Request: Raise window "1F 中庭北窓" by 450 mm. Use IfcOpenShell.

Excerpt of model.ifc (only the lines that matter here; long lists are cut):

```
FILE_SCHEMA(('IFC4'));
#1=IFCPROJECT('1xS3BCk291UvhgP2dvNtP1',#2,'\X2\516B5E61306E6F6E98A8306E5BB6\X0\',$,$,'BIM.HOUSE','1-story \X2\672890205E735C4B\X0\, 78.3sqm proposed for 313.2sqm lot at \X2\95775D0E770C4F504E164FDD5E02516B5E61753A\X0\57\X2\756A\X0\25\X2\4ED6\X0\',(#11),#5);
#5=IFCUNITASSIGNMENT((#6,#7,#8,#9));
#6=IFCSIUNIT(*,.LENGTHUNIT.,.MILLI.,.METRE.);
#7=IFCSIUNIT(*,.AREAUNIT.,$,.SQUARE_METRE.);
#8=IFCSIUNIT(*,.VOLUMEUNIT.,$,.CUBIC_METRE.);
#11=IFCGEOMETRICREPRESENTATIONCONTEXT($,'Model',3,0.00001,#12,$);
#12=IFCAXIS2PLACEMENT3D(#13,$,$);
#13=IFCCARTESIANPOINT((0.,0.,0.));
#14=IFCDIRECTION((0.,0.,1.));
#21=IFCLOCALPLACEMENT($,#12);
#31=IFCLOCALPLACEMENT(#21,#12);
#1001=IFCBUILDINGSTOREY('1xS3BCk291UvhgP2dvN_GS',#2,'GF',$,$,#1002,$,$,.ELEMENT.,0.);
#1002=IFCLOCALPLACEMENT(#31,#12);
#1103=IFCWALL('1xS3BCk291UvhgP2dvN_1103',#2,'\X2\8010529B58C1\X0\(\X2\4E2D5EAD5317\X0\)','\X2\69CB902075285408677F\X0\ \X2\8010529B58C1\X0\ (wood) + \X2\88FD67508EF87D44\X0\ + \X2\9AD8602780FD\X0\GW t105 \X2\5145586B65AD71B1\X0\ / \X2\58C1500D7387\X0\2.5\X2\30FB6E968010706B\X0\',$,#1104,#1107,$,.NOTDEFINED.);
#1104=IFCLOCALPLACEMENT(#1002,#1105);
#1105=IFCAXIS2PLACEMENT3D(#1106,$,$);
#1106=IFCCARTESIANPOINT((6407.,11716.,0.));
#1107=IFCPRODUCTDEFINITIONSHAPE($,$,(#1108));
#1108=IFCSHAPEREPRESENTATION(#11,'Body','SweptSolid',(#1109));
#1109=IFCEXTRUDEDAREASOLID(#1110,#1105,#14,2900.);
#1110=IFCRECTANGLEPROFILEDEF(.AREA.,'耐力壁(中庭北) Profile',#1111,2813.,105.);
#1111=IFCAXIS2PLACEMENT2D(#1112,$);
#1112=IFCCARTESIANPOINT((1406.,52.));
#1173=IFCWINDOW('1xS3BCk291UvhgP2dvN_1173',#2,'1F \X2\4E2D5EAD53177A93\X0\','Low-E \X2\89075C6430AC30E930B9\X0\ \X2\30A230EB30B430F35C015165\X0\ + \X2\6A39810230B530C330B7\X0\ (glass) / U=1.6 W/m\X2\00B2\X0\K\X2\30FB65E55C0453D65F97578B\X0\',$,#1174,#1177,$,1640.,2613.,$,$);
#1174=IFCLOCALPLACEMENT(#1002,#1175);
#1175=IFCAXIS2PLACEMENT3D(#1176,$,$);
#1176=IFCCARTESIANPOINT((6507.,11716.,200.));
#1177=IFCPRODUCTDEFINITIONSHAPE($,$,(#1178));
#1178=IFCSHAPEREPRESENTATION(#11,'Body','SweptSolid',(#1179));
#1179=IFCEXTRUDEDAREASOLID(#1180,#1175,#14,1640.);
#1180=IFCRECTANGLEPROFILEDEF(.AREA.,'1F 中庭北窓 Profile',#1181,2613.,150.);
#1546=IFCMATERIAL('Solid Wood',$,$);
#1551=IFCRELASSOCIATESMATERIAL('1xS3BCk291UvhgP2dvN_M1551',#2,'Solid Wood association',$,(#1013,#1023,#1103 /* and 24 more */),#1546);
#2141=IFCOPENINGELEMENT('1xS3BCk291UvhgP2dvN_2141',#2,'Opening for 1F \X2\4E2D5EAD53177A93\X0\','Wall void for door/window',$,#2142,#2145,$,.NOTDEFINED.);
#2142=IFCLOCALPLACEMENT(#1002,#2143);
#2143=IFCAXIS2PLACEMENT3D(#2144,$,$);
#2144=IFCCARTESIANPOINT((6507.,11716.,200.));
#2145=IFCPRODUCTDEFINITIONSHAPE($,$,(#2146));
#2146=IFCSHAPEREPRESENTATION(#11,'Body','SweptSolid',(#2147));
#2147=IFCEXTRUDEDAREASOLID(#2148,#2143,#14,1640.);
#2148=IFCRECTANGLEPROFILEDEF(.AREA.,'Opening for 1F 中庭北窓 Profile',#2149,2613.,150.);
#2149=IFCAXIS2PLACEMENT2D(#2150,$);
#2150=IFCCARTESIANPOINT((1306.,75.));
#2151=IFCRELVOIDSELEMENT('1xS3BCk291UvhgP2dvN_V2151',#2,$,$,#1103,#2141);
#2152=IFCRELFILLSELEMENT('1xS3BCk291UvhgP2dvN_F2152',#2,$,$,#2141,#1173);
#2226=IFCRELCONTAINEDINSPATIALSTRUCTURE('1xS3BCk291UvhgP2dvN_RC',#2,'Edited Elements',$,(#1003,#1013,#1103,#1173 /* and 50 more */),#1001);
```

```python
import numpy as np
import ifcopenshell
import ifcopenshell.api.geometry
import ifcopenshell.util.placement
import ifcopenshell.util.unit

model = ifcopenshell.open("model.ifc")
unit_scale = ifcopenshell.util.unit.calculate_unit_scale(model)

window = model.by_id(1173)
opening = window.FillsVoids[0].RelatingOpeningElement
dz = 0.45 / unit_scale

shift = np.array([0.0, 0.0, dz])
# The window is not placed relative to its opening, so move both.
for product in (opening, window):
    matrix = ifcopenshell.util.placement.get_local_placement(product.ObjectPlacement)
    matrix[:3, 3] += shift
    ifcopenshell.api.geometry.edit_object_placement(model, product=product, matrix=matrix, is_si=False)

print(f"moved by {dz * unit_scale:+.3f} m")

model.write("model_v2.ifc")
```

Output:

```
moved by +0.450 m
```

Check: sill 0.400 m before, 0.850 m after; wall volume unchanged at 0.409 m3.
